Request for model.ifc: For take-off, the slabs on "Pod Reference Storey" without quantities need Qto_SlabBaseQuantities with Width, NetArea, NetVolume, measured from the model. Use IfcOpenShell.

First a look at what the model holds.

```python
import ifcopenshell
import ifcopenshell.util.element
import ifcopenshell.util.unit

model = ifcopenshell.open("model.ifc")
print(model.schema)
for unit_type in ("LENGTHUNIT", "AREAUNIT", "VOLUMEUNIT"):
    print(unit_type, ifcopenshell.util.unit.calculate_unit_scale(model, unit_type))
storey = next(s for s in model.by_type("IfcBuildingStorey") if s.Name == "Pod Reference Storey")
slabs = [e for e in ifcopenshell.util.element.get_decomposition(storey) if e.is_a("IfcSlab")]
for e in sorted(slabs, key=lambda e: e.id()):
    print(e.id(), e.is_a(), e.Name, list(ifcopenshell.util.element.get_psets(e, qtos_only=True)), sep=" | ")
```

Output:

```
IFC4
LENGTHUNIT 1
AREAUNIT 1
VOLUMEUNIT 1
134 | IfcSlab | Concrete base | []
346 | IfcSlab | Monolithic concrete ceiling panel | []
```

```python
import ifcopenshell
import ifcopenshell.api.pset
import ifcopenshell.geom
import ifcopenshell.util.element
import ifcopenshell.util.shape
import ifcopenshell.util.unit

model = ifcopenshell.open("model.ifc")
unit_scale = ifcopenshell.util.unit.calculate_unit_scale(model)
area_scale = ifcopenshell.util.unit.calculate_unit_scale(model, "AREAUNIT")
volume_scale = ifcopenshell.util.unit.calculate_unit_scale(model, "VOLUMEUNIT")
settings = ifcopenshell.geom.settings()

storey = next(s for s in model.by_type("IfcBuildingStorey") if s.Name == "Pod Reference Storey")
slabs = [e for e in ifcopenshell.util.element.get_decomposition(storey) if e.is_a("IfcSlab")]

for e in sorted(slabs, key=lambda e: e.id()):
    if ifcopenshell.util.element.get_psets(e, qtos_only=True, should_inherit=False):
        continue
    # Geometry comes back in metres, in the element's own axes.
    shape = ifcopenshell.geom.create_shape(settings, e)
    values = {
        "Width": ifcopenshell.util.shape.get_z(shape.geometry) / unit_scale,
        "NetArea": ifcopenshell.util.shape.get_footprint_area(shape.geometry) / area_scale,
        "NetVolume": ifcopenshell.util.shape.get_volume(shape.geometry) / volume_scale,
    }
    qto = ifcopenshell.api.pset.add_qto(model, product=e, name="Qto_SlabBaseQuantities")
    ifcopenshell.api.pset.edit_qto(model, qto=qto, properties=values)
    print(e.id(), {k: round(v, 3) for k, v in values.items()})

model.write("model_edited.ifc")
```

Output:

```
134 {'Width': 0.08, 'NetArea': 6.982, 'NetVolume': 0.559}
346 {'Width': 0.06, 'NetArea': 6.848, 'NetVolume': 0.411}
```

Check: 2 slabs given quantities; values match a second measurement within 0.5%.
